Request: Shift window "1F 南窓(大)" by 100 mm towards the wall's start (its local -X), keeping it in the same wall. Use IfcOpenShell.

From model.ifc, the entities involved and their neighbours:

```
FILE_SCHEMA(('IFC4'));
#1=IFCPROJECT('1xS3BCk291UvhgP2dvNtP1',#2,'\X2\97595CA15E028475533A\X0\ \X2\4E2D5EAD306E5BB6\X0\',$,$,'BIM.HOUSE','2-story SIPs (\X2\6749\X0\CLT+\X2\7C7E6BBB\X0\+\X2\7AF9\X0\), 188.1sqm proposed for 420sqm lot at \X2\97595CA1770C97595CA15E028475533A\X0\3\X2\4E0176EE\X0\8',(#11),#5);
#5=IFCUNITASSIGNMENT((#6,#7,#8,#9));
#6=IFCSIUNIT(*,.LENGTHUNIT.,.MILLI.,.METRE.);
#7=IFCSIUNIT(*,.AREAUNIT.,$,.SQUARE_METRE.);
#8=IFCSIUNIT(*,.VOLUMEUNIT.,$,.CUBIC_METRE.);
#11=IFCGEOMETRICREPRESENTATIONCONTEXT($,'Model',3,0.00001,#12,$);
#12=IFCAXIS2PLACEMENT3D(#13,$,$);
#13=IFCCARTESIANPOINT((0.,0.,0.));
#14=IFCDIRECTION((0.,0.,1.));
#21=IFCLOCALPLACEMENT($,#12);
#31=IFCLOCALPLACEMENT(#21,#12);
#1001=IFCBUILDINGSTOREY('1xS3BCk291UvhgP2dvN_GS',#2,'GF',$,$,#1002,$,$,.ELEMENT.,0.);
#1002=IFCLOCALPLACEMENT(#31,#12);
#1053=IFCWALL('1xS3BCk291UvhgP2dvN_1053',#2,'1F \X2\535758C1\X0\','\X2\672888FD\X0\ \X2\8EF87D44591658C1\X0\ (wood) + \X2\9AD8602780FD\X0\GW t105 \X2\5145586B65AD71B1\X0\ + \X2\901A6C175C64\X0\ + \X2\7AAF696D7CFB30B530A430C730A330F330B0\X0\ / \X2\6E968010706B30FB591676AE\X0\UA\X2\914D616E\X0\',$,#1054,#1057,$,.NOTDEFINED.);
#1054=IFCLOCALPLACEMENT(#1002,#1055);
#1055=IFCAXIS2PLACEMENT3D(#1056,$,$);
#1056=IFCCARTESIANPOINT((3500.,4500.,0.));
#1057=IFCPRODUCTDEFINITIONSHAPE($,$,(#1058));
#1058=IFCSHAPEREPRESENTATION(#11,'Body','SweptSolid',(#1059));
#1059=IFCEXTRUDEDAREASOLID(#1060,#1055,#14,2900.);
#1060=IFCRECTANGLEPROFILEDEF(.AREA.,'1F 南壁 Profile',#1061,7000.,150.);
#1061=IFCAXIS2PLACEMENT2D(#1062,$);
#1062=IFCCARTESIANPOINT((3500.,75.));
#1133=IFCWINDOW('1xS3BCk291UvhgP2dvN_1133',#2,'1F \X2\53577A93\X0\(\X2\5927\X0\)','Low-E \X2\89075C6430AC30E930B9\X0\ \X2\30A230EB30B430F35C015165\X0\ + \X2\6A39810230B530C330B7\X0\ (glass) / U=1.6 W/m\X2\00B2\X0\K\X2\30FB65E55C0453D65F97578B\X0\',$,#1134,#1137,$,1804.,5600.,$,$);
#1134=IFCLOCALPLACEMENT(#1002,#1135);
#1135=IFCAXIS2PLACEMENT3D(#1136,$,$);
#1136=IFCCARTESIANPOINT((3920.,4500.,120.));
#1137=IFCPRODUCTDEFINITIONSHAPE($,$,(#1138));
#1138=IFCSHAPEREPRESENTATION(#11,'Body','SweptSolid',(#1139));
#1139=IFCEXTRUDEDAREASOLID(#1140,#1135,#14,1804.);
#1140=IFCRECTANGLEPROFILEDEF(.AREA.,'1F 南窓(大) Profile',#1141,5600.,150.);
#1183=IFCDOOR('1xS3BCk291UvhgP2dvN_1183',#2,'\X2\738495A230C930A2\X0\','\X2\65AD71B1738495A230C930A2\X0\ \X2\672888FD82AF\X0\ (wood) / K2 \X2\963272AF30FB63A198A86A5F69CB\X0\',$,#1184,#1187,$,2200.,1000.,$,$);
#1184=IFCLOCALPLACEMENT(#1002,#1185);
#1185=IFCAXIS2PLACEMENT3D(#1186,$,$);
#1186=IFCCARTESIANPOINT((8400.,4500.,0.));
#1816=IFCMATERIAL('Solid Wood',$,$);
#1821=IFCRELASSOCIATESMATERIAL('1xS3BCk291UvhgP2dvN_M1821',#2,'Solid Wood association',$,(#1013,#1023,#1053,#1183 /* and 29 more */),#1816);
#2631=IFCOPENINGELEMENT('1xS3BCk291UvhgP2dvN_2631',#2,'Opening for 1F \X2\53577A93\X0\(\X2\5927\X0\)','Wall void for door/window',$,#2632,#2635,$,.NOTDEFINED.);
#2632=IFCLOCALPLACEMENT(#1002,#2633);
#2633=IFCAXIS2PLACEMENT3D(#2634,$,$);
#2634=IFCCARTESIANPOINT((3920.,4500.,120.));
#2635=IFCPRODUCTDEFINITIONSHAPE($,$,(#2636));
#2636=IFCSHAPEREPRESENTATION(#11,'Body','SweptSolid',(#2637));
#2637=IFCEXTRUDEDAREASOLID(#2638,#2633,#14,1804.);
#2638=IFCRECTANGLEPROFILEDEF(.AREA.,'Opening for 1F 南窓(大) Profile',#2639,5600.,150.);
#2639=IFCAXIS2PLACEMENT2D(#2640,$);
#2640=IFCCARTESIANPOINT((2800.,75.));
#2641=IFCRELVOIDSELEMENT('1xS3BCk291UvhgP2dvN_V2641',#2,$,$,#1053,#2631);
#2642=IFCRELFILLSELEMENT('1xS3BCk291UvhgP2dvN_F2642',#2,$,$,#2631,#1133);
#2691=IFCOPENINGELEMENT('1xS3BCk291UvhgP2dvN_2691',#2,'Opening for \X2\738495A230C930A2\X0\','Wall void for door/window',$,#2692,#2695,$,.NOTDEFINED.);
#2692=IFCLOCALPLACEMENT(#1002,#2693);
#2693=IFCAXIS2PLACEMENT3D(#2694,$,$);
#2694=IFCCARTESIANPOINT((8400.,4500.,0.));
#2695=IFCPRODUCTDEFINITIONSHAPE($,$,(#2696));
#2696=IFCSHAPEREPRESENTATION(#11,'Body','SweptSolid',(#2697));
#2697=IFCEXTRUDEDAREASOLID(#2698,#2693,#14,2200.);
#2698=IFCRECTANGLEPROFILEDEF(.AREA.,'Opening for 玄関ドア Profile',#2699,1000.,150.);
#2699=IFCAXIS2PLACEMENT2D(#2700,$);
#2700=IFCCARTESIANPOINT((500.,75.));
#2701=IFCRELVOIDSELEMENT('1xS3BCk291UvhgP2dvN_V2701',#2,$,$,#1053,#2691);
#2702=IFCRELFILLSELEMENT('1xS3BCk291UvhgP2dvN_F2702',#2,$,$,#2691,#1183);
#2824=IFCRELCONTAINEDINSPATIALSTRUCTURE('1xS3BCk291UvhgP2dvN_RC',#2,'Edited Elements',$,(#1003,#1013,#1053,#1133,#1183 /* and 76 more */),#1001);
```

```python
import ifcopenshell
import ifcopenshell.api.geometry
import ifcopenshell.util.placement
import ifcopenshell.util.unit

model = ifcopenshell.open("model.ifc")
unit_scale = ifcopenshell.util.unit.calculate_unit_scale(model)

window = model.by_guid("1xS3BCk291UvhgP2dvN_1133")
opening = window.FillsVoids[0].RelatingOpeningElement
wall = opening.VoidsElements[0].RelatingBuildingElement

wall_matrix = ifcopenshell.util.placement.get_local_placement(wall.ObjectPlacement)
shift = wall_matrix[:3, 0] * -0.1 / unit_scale
before = ifcopenshell.util.placement.get_local_placement(window.ObjectPlacement)[:3, 3].copy()

# The window is not placed relative to its opening, so move both.
for product in (opening, window):
    matrix = ifcopenshell.util.placement.get_local_placement(product.ObjectPlacement)
    matrix[:3, 3] += shift
    ifcopenshell.api.geometry.edit_object_placement(model, product=product, matrix=matrix, is_si=False)

after = ifcopenshell.util.placement.get_local_placement(window.ObjectPlacement)[:3, 3]
print("window moved by", (after - before).round(3) + 0.0)

model.write("model_updated.ifc")
```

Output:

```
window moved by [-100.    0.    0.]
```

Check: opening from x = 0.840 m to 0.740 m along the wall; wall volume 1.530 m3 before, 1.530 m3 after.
